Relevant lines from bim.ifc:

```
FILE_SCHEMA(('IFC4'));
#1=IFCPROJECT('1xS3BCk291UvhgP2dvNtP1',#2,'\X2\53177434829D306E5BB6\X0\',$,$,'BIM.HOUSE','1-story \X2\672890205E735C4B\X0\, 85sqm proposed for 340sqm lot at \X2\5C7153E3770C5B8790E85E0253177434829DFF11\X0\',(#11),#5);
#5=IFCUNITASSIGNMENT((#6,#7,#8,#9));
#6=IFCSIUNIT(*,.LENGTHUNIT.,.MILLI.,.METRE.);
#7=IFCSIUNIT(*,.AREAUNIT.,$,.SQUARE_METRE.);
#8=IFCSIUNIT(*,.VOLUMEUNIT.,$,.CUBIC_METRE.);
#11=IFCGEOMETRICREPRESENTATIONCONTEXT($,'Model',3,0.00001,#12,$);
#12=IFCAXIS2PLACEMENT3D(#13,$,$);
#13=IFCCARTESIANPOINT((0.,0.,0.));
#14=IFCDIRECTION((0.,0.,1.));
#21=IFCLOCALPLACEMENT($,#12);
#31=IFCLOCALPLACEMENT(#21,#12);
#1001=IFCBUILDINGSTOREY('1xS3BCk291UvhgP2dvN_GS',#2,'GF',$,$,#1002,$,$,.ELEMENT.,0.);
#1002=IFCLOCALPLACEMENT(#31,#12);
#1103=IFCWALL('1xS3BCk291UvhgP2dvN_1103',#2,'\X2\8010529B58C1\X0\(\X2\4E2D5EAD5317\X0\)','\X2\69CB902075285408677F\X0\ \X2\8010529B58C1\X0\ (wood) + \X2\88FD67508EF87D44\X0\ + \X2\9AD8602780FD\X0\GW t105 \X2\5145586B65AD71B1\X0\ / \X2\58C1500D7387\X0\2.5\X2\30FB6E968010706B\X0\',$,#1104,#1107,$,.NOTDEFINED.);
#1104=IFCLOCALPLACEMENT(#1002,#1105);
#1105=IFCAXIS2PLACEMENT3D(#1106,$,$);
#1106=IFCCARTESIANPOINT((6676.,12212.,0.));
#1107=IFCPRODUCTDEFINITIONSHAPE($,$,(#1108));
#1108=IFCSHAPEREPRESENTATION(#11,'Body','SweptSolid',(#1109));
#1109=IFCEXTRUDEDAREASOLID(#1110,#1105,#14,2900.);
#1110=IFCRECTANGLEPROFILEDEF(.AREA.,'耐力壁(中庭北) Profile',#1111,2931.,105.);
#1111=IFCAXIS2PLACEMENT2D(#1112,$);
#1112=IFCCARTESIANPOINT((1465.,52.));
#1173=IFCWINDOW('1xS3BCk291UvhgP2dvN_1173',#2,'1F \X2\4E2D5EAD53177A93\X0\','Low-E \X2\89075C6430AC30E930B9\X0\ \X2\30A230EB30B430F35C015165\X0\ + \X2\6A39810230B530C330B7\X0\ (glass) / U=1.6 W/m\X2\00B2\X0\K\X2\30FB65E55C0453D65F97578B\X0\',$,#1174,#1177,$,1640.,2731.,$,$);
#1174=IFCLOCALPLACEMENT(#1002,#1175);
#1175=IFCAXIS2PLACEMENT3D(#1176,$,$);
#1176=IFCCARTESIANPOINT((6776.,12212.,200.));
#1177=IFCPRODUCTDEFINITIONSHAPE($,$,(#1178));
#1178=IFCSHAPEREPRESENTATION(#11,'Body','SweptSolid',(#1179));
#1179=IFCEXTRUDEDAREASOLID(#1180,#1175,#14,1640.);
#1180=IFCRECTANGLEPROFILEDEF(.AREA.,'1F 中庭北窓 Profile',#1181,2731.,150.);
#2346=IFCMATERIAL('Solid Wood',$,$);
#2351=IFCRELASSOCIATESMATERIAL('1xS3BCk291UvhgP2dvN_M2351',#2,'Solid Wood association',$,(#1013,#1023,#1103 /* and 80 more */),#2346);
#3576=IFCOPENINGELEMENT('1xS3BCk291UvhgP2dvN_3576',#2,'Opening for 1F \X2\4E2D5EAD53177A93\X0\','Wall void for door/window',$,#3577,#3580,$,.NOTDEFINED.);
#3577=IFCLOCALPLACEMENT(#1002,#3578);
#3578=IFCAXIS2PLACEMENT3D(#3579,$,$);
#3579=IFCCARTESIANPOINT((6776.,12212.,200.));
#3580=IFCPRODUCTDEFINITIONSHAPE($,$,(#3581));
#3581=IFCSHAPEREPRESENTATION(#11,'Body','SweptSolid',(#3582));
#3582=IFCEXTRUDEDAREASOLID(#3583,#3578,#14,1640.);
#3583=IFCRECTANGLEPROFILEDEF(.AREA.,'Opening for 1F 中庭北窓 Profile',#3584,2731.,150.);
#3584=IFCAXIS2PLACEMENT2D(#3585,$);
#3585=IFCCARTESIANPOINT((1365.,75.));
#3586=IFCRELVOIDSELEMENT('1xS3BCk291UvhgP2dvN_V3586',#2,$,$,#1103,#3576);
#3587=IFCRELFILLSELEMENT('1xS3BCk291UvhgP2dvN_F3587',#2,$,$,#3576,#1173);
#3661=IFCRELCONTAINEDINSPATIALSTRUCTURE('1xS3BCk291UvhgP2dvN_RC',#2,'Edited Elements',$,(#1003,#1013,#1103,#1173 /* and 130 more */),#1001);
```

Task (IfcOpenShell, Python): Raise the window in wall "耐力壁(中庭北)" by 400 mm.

```python
import numpy as np
import ifcopenshell
import ifcopenshell.api.geometry
import ifcopenshell.util.placement
import ifcopenshell.util.unit

model = ifcopenshell.open("bim.ifc")
unit_scale = ifcopenshell.util.unit.calculate_unit_scale(model)

window = model.by_guid("1xS3BCk291UvhgP2dvN_1173")
opening = window.FillsVoids[0].RelatingOpeningElement
dz = 0.4 / unit_scale

shift = np.array([0.0, 0.0, dz])
# The window is not placed relative to its opening, so move both.
for product in (opening, window):
    matrix = ifcopenshell.util.placement.get_local_placement(product.ObjectPlacement)
    matrix[:3, 3] += shift
    ifcopenshell.api.geometry.edit_object_placement(model, product=product, matrix=matrix, is_si=False)

print(f"moved by {dz * unit_scale:+.3f} m")

model.write("bim_updated.ifc")
```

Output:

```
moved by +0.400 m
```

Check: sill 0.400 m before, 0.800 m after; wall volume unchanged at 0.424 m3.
